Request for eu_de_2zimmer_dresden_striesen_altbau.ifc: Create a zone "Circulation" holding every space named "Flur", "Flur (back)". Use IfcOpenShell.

First a look at what the model holds.

```python
import ifcopenshell

model = ifcopenshell.open("eu_de_2zimmer_dresden_striesen_altbau.ifc")
print(model.schema)
seen = {}
for space in model.by_type("IfcSpace"):
    seen[space.LongName] = seen.get(space.LongName, 0) + 1
for name, count in sorted(seen.items(), key=str):
    print(count, "x", name)
print("zones:", [z.Name for z in model.by_type("IfcZone")][:20])
```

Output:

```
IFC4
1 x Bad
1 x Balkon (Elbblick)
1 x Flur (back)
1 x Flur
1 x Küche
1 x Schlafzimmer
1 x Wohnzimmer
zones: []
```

```python
import ifcopenshell
import ifcopenshell.api.group
import ifcopenshell.api.root

model = ifcopenshell.open("eu_de_2zimmer_dresden_striesen_altbau.ifc")

names = {"Flur", "Flur (back)"}
spaces = [s for s in model.by_type("IfcSpace") if s.LongName in names]

zone = ifcopenshell.api.root.create_entity(model, ifc_class="IfcZone", name="Circulation")
ifcopenshell.api.group.assign_group(model, products=spaces, group=zone)
print(len(spaces), "spaces in", zone.Name)

model.write("eu_de_2zimmer_dresden_striesen_altbau_edited.ifc")
```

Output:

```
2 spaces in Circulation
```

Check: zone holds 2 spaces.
